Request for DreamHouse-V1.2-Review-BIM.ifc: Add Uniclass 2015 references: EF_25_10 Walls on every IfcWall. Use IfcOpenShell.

First a look at what the model holds.

```python
import ifcopenshell

model = ifcopenshell.open("DreamHouse-V1.2-Review-BIM.ifc")
print(model.schema)
print("classifications:", [c.Name for c in model.by_type("IfcClassification")])
for ifc_class in ("IfcDoor", "IfcRoof", "IfcStair", "IfcWall", "IfcWindow"):
    print(ifc_class, len(model.by_type(ifc_class)))
```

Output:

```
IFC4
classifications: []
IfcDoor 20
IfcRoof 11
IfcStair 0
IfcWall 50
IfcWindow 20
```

```python
import ifcopenshell
import ifcopenshell.api.classification

model = ifcopenshell.open("DreamHouse-V1.2-Review-BIM.ifc")

system = ifcopenshell.api.classification.add_classification(model, classification="Uniclass 2015")

codes = {
    "IfcWall": ("EF_25_10", "Walls"),
}
for ifc_class, (code, name) in codes.items():
    products = model.by_type(ifc_class)
    ifcopenshell.api.classification.add_reference(
        model, products=products, classification=system, identification=code, name=name
    )
    print(code, len(products))

model.write("DreamHouse-V1.2-Review-BIM_rev.ifc")
```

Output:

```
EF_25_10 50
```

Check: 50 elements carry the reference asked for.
